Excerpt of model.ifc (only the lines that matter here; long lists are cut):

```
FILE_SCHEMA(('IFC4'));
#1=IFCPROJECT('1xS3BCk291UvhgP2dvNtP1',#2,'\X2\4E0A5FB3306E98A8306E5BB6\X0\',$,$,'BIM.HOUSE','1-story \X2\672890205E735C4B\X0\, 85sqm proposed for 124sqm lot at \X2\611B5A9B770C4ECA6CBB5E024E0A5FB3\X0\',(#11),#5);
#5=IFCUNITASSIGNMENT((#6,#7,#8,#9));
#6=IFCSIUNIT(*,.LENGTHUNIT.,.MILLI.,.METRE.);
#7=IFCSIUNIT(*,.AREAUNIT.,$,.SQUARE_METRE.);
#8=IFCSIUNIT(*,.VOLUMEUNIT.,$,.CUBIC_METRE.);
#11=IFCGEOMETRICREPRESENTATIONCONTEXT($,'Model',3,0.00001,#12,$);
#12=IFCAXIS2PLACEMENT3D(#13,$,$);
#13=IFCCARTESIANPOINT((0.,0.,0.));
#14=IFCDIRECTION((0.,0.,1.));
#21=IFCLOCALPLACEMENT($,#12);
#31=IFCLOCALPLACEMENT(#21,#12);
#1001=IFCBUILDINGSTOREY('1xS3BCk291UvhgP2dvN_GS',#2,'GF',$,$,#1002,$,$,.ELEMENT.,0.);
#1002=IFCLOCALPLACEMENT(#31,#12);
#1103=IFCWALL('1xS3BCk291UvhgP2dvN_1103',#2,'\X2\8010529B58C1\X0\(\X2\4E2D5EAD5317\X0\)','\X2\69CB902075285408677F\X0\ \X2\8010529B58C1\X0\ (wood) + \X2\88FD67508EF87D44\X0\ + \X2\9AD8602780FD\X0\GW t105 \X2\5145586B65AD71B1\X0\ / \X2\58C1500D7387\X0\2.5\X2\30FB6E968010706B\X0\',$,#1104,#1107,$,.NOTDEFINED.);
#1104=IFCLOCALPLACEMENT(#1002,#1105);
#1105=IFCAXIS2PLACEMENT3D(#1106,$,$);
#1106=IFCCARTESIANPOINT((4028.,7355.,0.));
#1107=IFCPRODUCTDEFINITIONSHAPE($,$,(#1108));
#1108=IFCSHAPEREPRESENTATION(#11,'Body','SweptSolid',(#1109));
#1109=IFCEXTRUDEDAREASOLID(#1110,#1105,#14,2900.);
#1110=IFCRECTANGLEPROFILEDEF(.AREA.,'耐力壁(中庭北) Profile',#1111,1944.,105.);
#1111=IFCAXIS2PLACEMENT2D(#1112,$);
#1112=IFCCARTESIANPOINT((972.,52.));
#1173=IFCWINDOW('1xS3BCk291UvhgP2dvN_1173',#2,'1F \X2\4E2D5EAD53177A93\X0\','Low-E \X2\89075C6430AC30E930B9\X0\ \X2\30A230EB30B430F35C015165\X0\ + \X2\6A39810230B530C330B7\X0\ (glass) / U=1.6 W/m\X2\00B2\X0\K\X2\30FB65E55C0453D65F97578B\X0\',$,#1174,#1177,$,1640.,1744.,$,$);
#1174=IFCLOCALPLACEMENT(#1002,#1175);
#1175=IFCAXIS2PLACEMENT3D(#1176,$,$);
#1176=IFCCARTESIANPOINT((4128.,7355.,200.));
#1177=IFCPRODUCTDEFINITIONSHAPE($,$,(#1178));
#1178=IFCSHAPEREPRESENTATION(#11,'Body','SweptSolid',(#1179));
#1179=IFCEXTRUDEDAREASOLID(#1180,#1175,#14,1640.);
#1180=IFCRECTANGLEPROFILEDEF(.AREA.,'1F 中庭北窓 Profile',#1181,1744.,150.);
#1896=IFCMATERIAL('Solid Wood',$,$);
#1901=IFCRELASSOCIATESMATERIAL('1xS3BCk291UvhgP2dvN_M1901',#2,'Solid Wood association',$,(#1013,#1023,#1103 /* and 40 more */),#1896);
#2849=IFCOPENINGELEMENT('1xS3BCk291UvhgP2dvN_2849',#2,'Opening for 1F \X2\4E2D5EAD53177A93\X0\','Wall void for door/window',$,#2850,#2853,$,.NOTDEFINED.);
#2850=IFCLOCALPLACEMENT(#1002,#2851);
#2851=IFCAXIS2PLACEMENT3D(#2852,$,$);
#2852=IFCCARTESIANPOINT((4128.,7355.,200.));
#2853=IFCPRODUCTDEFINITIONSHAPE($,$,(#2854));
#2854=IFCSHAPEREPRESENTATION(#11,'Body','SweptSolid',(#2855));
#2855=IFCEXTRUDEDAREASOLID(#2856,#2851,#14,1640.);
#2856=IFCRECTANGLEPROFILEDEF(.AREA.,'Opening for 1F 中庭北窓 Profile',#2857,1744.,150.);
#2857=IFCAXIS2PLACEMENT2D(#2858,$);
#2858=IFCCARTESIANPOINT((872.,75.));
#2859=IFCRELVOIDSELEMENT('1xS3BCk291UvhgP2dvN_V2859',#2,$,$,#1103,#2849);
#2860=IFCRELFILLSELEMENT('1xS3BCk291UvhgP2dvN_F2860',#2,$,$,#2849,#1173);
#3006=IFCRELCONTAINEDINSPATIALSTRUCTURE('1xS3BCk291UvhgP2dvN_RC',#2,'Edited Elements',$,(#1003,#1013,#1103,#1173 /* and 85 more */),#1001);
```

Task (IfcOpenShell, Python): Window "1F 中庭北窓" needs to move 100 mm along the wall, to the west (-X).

```python
import ifcopenshell
import ifcopenshell.api.geometry
import ifcopenshell.util.placement
import ifcopenshell.util.unit

model = ifcopenshell.open("model.ifc")
unit_scale = ifcopenshell.util.unit.calculate_unit_scale(model)

window = model.by_guid("1xS3BCk291UvhgP2dvN_1173")
opening = window.FillsVoids[0].RelatingOpeningElement
wall = opening.VoidsElements[0].RelatingBuildingElement

wall_matrix = ifcopenshell.util.placement.get_local_placement(wall.ObjectPlacement)
shift = wall_matrix[:3, 0] * -0.1 / unit_scale
before = ifcopenshell.util.placement.get_local_placement(window.ObjectPlacement)[:3, 3].copy()

# The window is not placed relative to its opening, so move both.
for product in (opening, window):
    matrix = ifcopenshell.util.placement.get_local_placement(product.ObjectPlacement)
    matrix[:3, 3] += shift
    ifcopenshell.api.geometry.edit_object_placement(model, product=product, matrix=matrix, is_si=False)

after = ifcopenshell.util.placement.get_local_placement(window.ObjectPlacement)[:3, 3]
print("window moved by", (after - before).round(3) + 0.0)

model.write("model_edited.ifc")
```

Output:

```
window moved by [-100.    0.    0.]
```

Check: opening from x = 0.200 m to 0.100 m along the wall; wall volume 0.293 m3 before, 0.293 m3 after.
